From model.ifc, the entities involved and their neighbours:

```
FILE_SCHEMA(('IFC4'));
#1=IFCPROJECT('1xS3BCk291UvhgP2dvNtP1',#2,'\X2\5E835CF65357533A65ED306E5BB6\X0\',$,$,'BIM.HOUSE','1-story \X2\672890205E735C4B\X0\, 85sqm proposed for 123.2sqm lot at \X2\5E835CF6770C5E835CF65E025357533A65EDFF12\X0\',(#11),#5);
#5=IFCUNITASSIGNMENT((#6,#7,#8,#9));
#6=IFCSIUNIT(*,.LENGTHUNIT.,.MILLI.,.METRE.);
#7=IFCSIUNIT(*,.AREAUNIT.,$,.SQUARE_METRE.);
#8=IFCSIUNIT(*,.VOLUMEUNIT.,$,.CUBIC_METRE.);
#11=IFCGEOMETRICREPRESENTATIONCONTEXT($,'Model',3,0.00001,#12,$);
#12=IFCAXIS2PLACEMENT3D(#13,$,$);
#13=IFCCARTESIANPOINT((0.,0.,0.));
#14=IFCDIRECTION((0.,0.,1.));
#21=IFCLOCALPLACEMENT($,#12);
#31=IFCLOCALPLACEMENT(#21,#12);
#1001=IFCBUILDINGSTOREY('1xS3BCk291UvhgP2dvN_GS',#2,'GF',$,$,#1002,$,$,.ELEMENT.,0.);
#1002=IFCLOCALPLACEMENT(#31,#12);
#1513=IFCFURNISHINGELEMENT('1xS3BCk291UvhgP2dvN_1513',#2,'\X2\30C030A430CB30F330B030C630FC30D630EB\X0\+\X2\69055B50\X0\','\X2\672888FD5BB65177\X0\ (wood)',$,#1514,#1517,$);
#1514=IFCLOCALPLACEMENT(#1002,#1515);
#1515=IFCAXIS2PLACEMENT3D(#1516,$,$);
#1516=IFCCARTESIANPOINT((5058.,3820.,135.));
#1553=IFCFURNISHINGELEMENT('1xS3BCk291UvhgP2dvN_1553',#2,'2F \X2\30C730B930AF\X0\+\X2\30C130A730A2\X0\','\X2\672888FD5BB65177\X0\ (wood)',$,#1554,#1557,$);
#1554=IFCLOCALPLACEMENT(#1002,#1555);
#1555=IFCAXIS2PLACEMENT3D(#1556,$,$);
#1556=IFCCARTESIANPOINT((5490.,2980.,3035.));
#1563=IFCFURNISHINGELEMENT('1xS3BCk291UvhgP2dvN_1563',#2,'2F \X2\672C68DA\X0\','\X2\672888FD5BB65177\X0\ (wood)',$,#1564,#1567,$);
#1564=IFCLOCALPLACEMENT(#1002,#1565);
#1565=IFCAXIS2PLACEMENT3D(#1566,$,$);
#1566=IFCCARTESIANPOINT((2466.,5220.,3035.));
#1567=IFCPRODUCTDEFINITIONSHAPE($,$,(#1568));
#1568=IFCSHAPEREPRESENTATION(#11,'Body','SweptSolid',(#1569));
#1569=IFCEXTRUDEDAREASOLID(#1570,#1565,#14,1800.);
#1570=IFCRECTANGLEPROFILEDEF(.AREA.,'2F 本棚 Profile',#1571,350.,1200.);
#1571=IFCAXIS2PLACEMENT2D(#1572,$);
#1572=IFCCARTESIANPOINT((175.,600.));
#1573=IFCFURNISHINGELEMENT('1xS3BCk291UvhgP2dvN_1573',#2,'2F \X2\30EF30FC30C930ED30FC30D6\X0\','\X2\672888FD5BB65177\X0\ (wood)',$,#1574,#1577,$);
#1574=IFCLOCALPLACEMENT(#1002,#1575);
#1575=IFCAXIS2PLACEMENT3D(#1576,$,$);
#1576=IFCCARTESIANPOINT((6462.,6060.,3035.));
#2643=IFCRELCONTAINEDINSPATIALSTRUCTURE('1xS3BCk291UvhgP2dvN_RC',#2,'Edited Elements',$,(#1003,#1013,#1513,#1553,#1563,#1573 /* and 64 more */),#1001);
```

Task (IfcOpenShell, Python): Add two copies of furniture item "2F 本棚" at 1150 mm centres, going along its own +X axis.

```python
import ifcopenshell
import ifcopenshell.api.geometry
import ifcopenshell.api.root
import ifcopenshell.util.element
import ifcopenshell.util.placement
import ifcopenshell.util.unit

model = ifcopenshell.open("model.ifc")
unit_scale = ifcopenshell.util.unit.calculate_unit_scale(model)


def reuse_history(source, copy):
    """copy_class also copies each property set's owner history, people and application; keep the originals."""
    for rel in copy.IsDefinedBy:
        if rel.is_a("IfcRelDefinesByProperties") and (history := rel.RelatingPropertyDefinition.OwnerHistory):
            rel.RelatingPropertyDefinition.OwnerHistory = source.OwnerHistory
            ifcopenshell.util.element.remove_deep2(model, history)


source = model.by_guid("1xS3BCk291UvhgP2dvN_1563")
base = ifcopenshell.util.placement.get_local_placement(source.ObjectPlacement)
step = base[:3, 0] * 1.15 / unit_scale

for i in range(1, 3):
    copy = ifcopenshell.api.root.copy_class(model, product=source)
    copy.Representation = ifcopenshell.util.element.copy_deep(
        model, source.Representation, exclude=["IfcGeometricRepresentationContext", "IfcRepresentationMap"]
    )
    reuse_history(source, copy)
    matrix = base.copy()
    matrix[:3, 3] += i * step
    print("added at", matrix[:3, 3].round(3) + 0.0)
    ifcopenshell.api.geometry.edit_object_placement(model, product=copy, matrix=matrix, is_si=False)

model.write("model_edited.ifc")
```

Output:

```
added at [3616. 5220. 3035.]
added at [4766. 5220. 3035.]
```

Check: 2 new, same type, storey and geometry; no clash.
